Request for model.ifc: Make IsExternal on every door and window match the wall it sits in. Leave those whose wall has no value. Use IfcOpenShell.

First a look at what the model holds.

```python
import ifcopenshell
import ifcopenshell.util.element

model = ifcopenshell.open("model.ifc")
print(model.schema)
seen = {}
for e in model.by_type("IfcDoor") + model.by_type("IfcWindow"):
    if not e.FillsVoids:
        continue
    host = e.FillsVoids[0].RelatingOpeningElement.VoidsElements[0].RelatingBuildingElement
    own = ifcopenshell.util.element.get_pset(e, f"Pset_{e.is_a()[3:].removesuffix('StandardCase')}Common", "IsExternal")
    wall = ifcopenshell.util.element.get_pset(host, "Pset_WallCommon", "IsExternal")
    seen[e.is_a(), own, wall] = seen.get((e.is_a(), own, wall), 0) + 1
for (cls, own, wall), count in sorted(seen.items(), key=str):
    print(count, cls, "IsExternal:", own, "| host wall:", wall)
```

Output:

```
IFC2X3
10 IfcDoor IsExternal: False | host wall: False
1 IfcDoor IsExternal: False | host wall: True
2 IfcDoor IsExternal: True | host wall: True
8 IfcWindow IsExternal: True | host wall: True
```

```python
import ifcopenshell
import ifcopenshell.api.pset
import ifcopenshell.util.element

model = ifcopenshell.open("model.ifc")

count = 0
for ifc_class, pset_name in (("IfcDoor", "Pset_DoorCommon"), ("IfcWindow", "Pset_WindowCommon")):
    for e in model.by_type(ifc_class):
        if not e.FillsVoids:
            continue
        host = e.FillsVoids[0].RelatingOpeningElement.VoidsElements[0].RelatingBuildingElement
        external = ifcopenshell.util.element.get_pset(host, "Pset_WallCommon", "IsExternal")
        if external is None or ifcopenshell.util.element.get_pset(e, pset_name, "IsExternal") == external:
            continue
        pset = ifcopenshell.api.pset.add_pset(model, product=e, name=pset_name)
        ifcopenshell.api.pset.edit_pset(model, pset=pset, properties={"IsExternal": external})
        count += 1

print(count, "updated")

model.write("model_updated.ifc")
```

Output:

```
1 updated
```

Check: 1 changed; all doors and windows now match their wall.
